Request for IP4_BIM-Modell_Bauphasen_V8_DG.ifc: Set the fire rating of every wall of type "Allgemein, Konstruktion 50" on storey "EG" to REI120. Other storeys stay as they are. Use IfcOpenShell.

First a look at what the model holds.

```python
import ifcopenshell
import ifcopenshell.util.element

model = ifcopenshell.open("IP4_BIM-Modell_Bauphasen_V8_DG.ifc")
print(model.schema)
storey = next(s for s in model.by_type("IfcBuildingStorey") if s.Name == "EG")
walls = [e for e in ifcopenshell.util.element.get_decomposition(storey) if e.is_a("IfcWall")]
seen = {}
for e in walls:
    element_type = ifcopenshell.util.element.get_type(e)
    key = (element_type.Name if element_type != e and element_type else None, ifcopenshell.util.element.get_pset(e, "Pset_WallCommon", "FireRating"))
    seen[key] = seen.get(key, 0) + 1
for (name, value), count in sorted(seen.items(), key=str):
    print(count, "x", name, "|", value)
```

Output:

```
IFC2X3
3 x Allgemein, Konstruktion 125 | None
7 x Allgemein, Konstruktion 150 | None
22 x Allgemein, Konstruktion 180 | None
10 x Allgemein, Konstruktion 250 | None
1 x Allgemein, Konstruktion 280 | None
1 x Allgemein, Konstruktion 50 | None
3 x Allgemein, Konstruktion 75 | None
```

```python
import ifcopenshell
import ifcopenshell.api.pset
import ifcopenshell.util.element

model = ifcopenshell.open("IP4_BIM-Modell_Bauphasen_V8_DG.ifc")

storey = next(s for s in model.by_type("IfcBuildingStorey") if s.Name == "EG")
walls = [e for e in ifcopenshell.util.element.get_decomposition(storey) if e.is_a("IfcWall")]

count = 0
for e in walls:
    element_type = ifcopenshell.util.element.get_type(e)
    if element_type in (None, e) or element_type.Name != "Allgemein, Konstruktion 50":
        continue
    # add_pset returns the element's existing set when there is one.
    pset = ifcopenshell.api.pset.add_pset(model, product=e, name="Pset_WallCommon")
    ifcopenshell.api.pset.edit_pset(model, pset=pset, properties={"FireRating": "REI120"})
    count += 1

print(count, "walls updated")

model.write("IP4_BIM-Modell_Bauphasen_V8_DG_v2.ifc")
```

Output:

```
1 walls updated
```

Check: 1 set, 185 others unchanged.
